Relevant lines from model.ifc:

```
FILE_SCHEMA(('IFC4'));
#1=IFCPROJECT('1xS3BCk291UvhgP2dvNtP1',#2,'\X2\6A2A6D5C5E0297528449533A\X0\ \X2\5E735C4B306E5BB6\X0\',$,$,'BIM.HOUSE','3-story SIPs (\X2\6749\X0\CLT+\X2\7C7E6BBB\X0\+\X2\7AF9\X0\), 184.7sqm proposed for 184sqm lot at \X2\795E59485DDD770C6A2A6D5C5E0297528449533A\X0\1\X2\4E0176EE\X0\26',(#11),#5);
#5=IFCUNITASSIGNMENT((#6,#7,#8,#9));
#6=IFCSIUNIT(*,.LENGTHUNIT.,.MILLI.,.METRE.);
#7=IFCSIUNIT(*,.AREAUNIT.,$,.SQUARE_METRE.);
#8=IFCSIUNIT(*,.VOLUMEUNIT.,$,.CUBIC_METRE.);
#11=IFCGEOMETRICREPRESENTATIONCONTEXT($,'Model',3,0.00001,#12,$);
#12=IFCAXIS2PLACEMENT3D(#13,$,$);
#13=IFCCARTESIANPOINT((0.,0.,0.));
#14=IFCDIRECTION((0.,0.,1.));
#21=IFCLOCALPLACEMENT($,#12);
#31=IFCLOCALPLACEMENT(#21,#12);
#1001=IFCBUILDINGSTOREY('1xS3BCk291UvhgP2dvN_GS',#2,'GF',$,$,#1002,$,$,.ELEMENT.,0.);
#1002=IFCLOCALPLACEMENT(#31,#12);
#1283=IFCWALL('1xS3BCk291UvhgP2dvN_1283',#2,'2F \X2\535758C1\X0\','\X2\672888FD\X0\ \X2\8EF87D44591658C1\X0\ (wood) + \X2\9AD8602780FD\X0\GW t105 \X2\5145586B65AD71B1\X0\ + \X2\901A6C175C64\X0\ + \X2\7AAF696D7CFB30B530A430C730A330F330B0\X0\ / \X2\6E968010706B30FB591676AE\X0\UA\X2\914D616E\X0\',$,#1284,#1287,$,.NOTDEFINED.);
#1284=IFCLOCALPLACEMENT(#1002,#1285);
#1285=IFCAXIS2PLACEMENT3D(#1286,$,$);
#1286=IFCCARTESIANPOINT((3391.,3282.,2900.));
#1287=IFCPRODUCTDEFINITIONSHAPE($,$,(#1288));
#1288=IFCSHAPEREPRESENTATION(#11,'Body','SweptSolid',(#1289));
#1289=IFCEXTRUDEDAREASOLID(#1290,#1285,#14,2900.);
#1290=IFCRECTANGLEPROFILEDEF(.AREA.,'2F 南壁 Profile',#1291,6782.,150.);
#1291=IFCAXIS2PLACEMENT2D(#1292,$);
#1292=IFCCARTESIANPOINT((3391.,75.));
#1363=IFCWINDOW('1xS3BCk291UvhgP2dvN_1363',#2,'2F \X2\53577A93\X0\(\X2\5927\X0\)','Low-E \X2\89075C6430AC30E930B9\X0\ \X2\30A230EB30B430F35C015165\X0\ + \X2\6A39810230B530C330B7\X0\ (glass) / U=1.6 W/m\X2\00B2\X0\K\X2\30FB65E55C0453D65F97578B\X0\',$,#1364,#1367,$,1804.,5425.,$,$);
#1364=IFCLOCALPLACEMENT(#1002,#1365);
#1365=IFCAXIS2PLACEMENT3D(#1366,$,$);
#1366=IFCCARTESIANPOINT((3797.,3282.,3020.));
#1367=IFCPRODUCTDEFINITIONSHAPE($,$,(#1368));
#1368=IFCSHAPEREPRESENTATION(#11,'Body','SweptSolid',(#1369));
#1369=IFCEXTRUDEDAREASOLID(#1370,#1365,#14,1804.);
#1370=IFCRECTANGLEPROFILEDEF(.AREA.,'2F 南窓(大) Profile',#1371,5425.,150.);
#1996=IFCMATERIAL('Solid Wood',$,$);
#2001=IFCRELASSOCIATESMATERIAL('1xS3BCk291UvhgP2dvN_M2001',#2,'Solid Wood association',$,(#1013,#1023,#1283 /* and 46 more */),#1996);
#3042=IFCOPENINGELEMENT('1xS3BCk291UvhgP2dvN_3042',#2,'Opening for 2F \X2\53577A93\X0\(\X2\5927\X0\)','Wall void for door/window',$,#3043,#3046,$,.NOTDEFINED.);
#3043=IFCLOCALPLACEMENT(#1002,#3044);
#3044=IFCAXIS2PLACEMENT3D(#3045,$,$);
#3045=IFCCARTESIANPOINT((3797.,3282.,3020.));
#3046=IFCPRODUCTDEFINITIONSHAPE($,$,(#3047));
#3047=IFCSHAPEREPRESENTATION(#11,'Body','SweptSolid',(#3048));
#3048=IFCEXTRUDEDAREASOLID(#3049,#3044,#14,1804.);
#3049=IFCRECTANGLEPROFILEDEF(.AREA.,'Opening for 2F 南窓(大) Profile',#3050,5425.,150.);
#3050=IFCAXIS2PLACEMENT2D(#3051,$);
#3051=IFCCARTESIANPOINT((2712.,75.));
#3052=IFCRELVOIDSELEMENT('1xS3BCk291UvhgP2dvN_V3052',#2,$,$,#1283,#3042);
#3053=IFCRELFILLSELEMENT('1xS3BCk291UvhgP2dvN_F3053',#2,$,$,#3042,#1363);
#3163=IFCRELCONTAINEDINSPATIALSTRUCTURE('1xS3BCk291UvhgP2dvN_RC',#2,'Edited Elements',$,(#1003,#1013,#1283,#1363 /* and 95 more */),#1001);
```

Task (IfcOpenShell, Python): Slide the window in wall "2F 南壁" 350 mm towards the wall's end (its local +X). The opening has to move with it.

```python
import ifcopenshell
import ifcopenshell.api.geometry
import ifcopenshell.util.placement

model = ifcopenshell.open("model.ifc")

window = model.by_guid("1xS3BCk291UvhgP2dvN_1363")
opening = window.FillsVoids[0].RelatingOpeningElement
wall = opening.VoidsElements[0].RelatingBuildingElement

wall_matrix = ifcopenshell.util.placement.get_local_placement(wall.ObjectPlacement)
shift = wall_matrix[:3, 0] * 350.0
before = ifcopenshell.util.placement.get_local_placement(window.ObjectPlacement)[:3, 3].copy()

# The window is not placed relative to its opening, so move both.
for product in (opening, window):
    matrix = ifcopenshell.util.placement.get_local_placement(product.ObjectPlacement)
    matrix[:3, 3] += shift
    ifcopenshell.api.geometry.edit_object_placement(model, product=product, matrix=matrix, is_si=False)

after = ifcopenshell.util.placement.get_local_placement(window.ObjectPlacement)[:3, 3]
print("window moved by", (after - before).round(3) + 0.0)

model.write("model_updated.ifc")
```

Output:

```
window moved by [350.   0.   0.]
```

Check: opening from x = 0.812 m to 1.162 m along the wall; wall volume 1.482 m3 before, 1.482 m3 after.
